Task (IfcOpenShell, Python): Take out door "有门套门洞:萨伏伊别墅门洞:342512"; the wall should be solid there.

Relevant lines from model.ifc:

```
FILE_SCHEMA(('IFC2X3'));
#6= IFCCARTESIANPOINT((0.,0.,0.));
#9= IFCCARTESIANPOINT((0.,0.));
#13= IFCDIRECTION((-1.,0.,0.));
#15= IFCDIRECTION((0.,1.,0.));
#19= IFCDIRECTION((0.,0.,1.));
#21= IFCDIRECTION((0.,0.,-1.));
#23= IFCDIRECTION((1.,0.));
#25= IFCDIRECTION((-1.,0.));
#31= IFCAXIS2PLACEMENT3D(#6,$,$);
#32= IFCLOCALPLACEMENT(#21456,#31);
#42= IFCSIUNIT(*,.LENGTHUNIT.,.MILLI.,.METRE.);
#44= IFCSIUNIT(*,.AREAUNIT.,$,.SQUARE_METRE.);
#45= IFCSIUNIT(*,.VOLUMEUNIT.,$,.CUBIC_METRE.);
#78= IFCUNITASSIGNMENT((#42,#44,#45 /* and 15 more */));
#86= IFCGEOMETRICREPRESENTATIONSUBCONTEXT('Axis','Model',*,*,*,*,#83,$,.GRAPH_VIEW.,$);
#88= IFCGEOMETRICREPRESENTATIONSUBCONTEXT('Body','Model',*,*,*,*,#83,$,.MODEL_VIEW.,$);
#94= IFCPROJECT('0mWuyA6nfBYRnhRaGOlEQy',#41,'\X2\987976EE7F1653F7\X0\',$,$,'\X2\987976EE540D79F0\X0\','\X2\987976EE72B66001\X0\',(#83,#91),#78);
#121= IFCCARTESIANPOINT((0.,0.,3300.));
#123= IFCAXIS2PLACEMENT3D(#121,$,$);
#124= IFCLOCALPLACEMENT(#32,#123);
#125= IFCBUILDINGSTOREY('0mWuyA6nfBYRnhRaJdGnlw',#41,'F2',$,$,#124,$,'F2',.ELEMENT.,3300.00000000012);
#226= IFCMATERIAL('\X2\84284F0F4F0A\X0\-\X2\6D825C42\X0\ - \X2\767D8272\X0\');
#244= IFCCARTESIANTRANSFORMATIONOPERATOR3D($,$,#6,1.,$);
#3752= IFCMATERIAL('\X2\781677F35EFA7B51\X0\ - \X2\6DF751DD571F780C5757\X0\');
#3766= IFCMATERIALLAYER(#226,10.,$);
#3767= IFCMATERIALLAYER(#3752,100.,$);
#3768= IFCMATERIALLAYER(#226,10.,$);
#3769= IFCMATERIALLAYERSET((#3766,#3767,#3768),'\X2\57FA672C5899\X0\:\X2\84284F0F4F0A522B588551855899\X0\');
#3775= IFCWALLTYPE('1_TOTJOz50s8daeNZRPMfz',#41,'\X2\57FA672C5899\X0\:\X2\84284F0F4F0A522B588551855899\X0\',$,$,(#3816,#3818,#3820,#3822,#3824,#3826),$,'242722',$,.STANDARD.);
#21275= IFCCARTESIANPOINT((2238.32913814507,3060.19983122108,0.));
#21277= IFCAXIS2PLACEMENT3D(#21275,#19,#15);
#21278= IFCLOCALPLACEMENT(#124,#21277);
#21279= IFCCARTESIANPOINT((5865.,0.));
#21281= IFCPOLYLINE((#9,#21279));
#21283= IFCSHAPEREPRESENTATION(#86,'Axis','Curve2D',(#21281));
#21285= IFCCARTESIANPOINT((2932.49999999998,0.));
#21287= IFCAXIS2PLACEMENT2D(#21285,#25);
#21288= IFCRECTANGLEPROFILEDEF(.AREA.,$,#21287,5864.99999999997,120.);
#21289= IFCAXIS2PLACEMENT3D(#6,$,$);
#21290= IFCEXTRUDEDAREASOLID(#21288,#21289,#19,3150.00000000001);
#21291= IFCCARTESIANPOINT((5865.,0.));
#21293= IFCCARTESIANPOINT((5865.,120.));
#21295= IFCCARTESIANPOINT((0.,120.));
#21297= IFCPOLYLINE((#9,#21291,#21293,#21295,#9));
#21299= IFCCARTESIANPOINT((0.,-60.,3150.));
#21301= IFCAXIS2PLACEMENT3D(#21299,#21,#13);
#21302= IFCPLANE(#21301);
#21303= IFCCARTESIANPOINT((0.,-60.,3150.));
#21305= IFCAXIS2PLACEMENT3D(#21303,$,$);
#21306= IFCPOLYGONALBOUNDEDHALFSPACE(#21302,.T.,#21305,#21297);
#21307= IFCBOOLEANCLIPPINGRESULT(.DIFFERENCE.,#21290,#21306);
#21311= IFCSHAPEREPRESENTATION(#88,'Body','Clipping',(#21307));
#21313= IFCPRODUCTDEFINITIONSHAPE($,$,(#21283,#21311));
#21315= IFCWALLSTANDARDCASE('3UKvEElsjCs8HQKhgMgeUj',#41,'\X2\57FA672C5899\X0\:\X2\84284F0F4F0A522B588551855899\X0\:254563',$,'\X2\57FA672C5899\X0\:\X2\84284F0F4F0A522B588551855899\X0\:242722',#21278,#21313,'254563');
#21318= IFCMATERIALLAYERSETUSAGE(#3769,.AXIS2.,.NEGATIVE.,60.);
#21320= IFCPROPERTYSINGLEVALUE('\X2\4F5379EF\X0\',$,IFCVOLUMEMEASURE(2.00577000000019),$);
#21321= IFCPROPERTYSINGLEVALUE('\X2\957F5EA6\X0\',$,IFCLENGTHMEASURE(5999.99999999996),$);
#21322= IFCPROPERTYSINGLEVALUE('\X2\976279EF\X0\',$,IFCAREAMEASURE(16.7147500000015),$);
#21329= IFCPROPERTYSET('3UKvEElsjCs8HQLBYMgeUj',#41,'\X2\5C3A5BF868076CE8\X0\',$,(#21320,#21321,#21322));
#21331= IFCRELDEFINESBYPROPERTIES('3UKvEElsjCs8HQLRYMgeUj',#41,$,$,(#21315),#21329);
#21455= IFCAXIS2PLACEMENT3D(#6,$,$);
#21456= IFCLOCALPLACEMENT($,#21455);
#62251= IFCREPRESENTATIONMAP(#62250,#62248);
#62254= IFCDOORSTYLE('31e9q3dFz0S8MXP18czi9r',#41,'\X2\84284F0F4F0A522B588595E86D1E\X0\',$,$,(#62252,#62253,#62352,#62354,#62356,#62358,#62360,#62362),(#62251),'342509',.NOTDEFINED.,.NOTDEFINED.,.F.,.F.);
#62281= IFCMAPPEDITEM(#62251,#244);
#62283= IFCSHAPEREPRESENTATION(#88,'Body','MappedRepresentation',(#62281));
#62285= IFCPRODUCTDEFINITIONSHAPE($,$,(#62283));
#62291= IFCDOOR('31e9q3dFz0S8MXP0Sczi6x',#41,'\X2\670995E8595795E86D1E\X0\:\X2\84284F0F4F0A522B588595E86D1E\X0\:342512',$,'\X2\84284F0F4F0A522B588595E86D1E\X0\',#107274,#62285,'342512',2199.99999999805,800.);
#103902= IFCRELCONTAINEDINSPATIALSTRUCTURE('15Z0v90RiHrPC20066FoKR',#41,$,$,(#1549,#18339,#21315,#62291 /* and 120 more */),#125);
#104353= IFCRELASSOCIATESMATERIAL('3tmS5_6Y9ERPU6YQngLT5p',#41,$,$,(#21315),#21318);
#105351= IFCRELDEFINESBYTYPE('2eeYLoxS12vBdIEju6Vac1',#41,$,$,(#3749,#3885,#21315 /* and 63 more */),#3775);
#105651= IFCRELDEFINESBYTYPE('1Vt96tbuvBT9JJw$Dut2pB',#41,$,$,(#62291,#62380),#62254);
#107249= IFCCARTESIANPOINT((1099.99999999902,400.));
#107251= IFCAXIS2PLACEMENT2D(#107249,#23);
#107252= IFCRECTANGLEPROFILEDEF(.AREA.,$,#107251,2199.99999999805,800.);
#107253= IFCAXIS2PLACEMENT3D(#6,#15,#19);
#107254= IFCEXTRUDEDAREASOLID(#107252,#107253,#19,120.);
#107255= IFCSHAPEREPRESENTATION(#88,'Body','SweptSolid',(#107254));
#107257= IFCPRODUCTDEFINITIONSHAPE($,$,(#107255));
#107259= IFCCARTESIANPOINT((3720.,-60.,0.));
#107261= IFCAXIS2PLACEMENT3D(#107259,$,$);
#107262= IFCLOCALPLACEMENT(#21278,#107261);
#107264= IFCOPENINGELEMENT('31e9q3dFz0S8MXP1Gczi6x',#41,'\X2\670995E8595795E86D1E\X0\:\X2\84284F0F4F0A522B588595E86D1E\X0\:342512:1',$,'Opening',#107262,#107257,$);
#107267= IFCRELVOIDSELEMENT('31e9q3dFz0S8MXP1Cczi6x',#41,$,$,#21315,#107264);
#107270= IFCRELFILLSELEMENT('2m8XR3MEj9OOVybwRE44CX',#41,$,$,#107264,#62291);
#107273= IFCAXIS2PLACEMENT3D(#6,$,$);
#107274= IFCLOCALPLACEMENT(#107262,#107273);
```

```python
import ifcopenshell
import ifcopenshell.api.feature
import ifcopenshell.api.pset
import ifcopenshell.api.root
import ifcopenshell.geom
import ifcopenshell.util.element
import ifcopenshell.util.shape
import ifcopenshell.util.unit

model = ifcopenshell.open("model.ifc")
area_scale = ifcopenshell.util.unit.calculate_unit_scale(model, "AREAUNIT")
volume_scale = ifcopenshell.util.unit.calculate_unit_scale(model, "VOLUMEUNIT")
settings = ifcopenshell.geom.settings()


def volume(element):
    """Net volume in cubic metres, openings subtracted."""
    shape = ifcopenshell.geom.create_shape(settings, element)
    return ifcopenshell.util.shape.get_volume(shape.geometry)


door = model.by_id(62291)
opening = door.FillsVoids[0].RelatingOpeningElement
wall = opening.VoidsElements[0].RelatingBuildingElement
before = volume(wall)

ifcopenshell.api.root.remove_product(model, product=door)
ifcopenshell.api.feature.remove_feature(model, feature=opening)

after = volume(wall)
thickness = 0.12  # wall thickness in metres

# Update the wall's stored quantities.
pset = model.by_id(ifcopenshell.util.element.get_pset(wall, "尺寸标注", should_inherit=False)["id"])
ifcopenshell.api.pset.edit_pset(model, pset=pset, properties={
    "体积": model.create_entity("IfcVolumeMeasure", after / volume_scale),
    "面积": model.create_entity("IfcAreaMeasure", after / thickness / area_scale),
})

print(f"wall volume {before:.3f} -> {after:.3f} m3")

model.write("model_updated.ifc")
```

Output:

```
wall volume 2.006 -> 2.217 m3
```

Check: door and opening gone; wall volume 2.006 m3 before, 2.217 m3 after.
